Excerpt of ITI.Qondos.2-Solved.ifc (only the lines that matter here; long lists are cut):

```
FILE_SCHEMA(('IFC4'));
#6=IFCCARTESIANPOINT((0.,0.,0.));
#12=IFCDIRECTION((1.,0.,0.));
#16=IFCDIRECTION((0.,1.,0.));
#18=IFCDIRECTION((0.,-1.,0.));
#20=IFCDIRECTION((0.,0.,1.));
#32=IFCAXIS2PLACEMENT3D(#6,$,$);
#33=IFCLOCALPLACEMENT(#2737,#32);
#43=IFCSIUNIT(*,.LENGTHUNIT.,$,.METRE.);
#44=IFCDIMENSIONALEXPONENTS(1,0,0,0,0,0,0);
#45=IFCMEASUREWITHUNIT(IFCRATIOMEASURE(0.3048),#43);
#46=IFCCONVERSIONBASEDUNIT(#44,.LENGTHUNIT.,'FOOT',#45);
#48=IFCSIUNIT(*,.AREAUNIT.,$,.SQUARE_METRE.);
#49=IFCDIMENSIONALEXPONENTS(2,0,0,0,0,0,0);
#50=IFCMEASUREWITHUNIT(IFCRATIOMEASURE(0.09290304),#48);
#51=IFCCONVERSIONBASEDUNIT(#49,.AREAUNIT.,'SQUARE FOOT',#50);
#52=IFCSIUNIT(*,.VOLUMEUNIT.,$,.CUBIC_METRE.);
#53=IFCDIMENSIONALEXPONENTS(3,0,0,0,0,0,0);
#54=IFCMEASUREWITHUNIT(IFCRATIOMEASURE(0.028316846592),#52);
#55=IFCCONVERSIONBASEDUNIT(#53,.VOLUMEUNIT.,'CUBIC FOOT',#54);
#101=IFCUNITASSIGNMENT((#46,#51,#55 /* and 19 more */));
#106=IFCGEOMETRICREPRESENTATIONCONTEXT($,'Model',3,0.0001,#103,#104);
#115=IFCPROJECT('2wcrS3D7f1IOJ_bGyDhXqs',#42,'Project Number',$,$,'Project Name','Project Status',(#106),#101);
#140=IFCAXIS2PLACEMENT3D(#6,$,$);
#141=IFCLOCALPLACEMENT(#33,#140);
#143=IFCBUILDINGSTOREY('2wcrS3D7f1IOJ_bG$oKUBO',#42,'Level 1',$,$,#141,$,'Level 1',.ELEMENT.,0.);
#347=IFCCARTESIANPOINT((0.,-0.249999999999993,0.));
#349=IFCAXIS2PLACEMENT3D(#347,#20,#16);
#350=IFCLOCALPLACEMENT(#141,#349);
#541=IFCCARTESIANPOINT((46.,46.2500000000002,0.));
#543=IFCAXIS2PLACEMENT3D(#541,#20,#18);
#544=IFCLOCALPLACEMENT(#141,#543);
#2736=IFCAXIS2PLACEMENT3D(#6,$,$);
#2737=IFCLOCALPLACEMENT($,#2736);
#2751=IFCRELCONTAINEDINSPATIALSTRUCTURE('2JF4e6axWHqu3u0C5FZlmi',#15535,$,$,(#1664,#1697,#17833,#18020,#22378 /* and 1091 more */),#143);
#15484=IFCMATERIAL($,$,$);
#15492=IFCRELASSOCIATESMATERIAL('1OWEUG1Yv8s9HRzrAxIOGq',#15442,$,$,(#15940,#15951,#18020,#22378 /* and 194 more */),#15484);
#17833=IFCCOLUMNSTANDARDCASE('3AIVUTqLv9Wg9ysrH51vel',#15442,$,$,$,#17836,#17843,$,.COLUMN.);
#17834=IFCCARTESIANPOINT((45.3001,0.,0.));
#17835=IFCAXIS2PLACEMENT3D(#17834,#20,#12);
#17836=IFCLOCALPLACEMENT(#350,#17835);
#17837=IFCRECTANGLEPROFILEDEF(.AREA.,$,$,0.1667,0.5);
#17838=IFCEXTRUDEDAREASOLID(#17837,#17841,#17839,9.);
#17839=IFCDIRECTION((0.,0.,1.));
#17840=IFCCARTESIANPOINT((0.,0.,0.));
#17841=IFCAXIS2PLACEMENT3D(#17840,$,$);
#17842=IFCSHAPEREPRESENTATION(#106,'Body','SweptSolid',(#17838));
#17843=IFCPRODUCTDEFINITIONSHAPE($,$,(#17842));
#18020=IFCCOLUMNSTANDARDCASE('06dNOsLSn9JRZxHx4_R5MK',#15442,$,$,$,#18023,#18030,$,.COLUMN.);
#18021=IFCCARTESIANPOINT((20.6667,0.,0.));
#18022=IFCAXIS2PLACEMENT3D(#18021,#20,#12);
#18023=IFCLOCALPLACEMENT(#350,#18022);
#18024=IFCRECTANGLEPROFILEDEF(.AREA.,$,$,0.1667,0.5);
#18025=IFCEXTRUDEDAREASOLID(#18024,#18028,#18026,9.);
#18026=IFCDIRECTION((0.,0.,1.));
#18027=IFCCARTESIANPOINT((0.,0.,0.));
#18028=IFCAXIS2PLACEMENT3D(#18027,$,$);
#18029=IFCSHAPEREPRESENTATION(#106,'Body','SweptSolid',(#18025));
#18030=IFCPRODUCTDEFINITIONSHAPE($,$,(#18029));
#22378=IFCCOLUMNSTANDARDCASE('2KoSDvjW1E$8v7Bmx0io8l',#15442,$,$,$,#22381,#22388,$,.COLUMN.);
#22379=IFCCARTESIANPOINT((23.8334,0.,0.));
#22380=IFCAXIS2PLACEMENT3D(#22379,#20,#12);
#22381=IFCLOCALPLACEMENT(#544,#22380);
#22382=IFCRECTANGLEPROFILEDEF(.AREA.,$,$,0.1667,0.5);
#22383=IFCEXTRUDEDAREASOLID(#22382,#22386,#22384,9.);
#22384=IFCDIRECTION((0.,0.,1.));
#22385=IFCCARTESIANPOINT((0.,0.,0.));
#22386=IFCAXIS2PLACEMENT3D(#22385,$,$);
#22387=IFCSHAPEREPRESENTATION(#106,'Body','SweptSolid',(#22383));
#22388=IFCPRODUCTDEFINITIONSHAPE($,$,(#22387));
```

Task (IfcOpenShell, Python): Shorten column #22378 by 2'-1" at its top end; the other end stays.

```python
import ifcopenshell
import ifcopenshell.util.unit

model = ifcopenshell.open("ITI.Qondos.2-Solved.ifc")
unit_scale = ifcopenshell.util.unit.calculate_unit_scale(model)

member = model.by_id(22378)
change = -25 * 0.0254 / unit_scale

# The extrusion runs towards the end named, so only its depth changes.
body = next(r for r in member.Representation.Representations if r.RepresentationIdentifier == "Body")
solid = body.Items[0]
old_length = solid.Depth
solid.Depth += change

print(f"length {old_length:g} -> {solid.Depth:g}")

model.write("ITI.Qondos.2-Solved_edited.ifc")
```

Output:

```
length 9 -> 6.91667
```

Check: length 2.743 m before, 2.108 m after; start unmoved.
